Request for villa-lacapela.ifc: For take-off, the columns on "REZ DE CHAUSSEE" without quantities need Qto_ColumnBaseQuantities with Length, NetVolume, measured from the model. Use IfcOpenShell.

First a look at what the model holds.

```python
import ifcopenshell
import ifcopenshell.util.element
import ifcopenshell.util.unit

model = ifcopenshell.open("villa-lacapela.ifc")
print(model.schema)
for unit_type in ("LENGTHUNIT", "AREAUNIT", "VOLUMEUNIT"):
    print(unit_type, ifcopenshell.util.unit.calculate_unit_scale(model, unit_type))
storey = next(s for s in model.by_type("IfcBuildingStorey") if s.Name == "REZ DE CHAUSSEE")
columns = [e for e in ifcopenshell.util.element.get_decomposition(storey) if e.is_a("IfcColumn")]
for e in sorted(columns, key=lambda e: e.id()):
    print(e.id(), e.is_a(), e.Name, list(ifcopenshell.util.element.get_psets(e, qtos_only=True)), sep=" | ")
```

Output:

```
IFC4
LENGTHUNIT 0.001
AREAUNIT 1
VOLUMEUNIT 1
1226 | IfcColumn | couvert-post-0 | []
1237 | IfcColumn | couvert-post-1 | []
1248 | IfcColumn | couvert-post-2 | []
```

```python
import ifcopenshell
import ifcopenshell.api.pset
import ifcopenshell.geom
import ifcopenshell.util.element
import ifcopenshell.util.shape
import ifcopenshell.util.unit

model = ifcopenshell.open("villa-lacapela.ifc")
unit_scale = ifcopenshell.util.unit.calculate_unit_scale(model)
volume_scale = ifcopenshell.util.unit.calculate_unit_scale(model, "VOLUMEUNIT")
settings = ifcopenshell.geom.settings()

storey = next(s for s in model.by_type("IfcBuildingStorey") if s.Name == "REZ DE CHAUSSEE")
columns = [e for e in ifcopenshell.util.element.get_decomposition(storey) if e.is_a("IfcColumn")]

for e in sorted(columns, key=lambda e: e.id()):
    if ifcopenshell.util.element.get_psets(e, qtos_only=True, should_inherit=False):
        continue
    # Geometry comes back in metres, in the element's own axes.
    shape = ifcopenshell.geom.create_shape(settings, e)
    values = {
        "Length": ifcopenshell.util.shape.get_z(shape.geometry) / unit_scale,
        "NetVolume": ifcopenshell.util.shape.get_volume(shape.geometry) / volume_scale,
    }
    qto = ifcopenshell.api.pset.add_qto(model, product=e, name="Qto_ColumnBaseQuantities")
    ifcopenshell.api.pset.edit_qto(model, qto=qto, properties=values)
    print(e.id(), {k: round(v, 3) for k, v in values.items()})

model.write("villa-lacapela_edited.ifc")
```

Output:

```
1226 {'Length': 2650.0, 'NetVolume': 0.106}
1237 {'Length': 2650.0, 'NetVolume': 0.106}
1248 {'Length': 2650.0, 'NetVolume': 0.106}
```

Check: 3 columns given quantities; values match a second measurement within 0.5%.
